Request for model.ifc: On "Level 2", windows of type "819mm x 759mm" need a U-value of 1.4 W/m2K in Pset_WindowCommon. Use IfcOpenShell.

First a look at what the model holds.

```python
import ifcopenshell
import ifcopenshell.util.element

model = ifcopenshell.open("model.ifc")
print(model.schema)
storey = next(s for s in model.by_type("IfcBuildingStorey") if s.Name == "Level 2")
windows = [e for e in ifcopenshell.util.element.get_decomposition(storey) if e.is_a("IfcWindow")]
seen = {}
for e in windows:
    element_type = ifcopenshell.util.element.get_type(e)
    key = (element_type.Name if element_type != e and element_type else None, ifcopenshell.util.element.get_pset(e, "Pset_WindowCommon", "ThermalTransmittance"))
    seen[key] = seen.get(key, 0) + 1
for (name, value), count in sorted(seen.items(), key=str):
    print(count, "x", name, "|", value)
```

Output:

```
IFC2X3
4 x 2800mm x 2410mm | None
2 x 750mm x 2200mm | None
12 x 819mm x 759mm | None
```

```python
import ifcopenshell
import ifcopenshell.api.pset
import ifcopenshell.util.element

model = ifcopenshell.open("model.ifc")

storey = next(s for s in model.by_type("IfcBuildingStorey") if s.Name == "Level 2")
windows = [e for e in ifcopenshell.util.element.get_decomposition(storey) if e.is_a("IfcWindow")]

count = 0
for e in windows:
    element_type = ifcopenshell.util.element.get_type(e)
    if element_type in (None, e) or element_type.Name != "819mm x 759mm":
        continue
    # add_pset returns the element's existing set when there is one.
    pset = ifcopenshell.api.pset.add_pset(model, product=e, name="Pset_WindowCommon")
    ifcopenshell.api.pset.edit_pset(model, pset=pset, properties={"ThermalTransmittance": 1.4})
    count += 1

print(count, "windows updated")

model.write("model_edited.ifc")
```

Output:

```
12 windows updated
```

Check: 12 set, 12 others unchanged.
